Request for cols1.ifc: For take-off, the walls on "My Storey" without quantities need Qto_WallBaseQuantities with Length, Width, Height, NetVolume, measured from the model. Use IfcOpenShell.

First a look at what the model holds.

```python
import ifcopenshell
import ifcopenshell.util.element
import ifcopenshell.util.unit

model = ifcopenshell.open("cols1.ifc")
print(model.schema)
for unit_type in ("LENGTHUNIT", "AREAUNIT", "VOLUMEUNIT"):
    print(unit_type, ifcopenshell.util.unit.calculate_unit_scale(model, unit_type))
storey = next(s for s in model.by_type("IfcBuildingStorey") if s.Name == "My Storey")
walls = [e for e in ifcopenshell.util.element.get_decomposition(storey) if e.is_a("IfcWall")]
for e in sorted(walls, key=lambda e: e.id()):
    print(e.id(), e.is_a(), e.Name, list(ifcopenshell.util.element.get_psets(e, qtos_only=True)), sep=" | ")
```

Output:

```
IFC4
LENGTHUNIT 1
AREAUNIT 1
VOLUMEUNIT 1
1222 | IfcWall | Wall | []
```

```python
import ifcopenshell
import ifcopenshell.api.pset
import ifcopenshell.geom
import ifcopenshell.util.element
import ifcopenshell.util.shape
import ifcopenshell.util.unit

model = ifcopenshell.open("cols1.ifc")
unit_scale = ifcopenshell.util.unit.calculate_unit_scale(model)
volume_scale = ifcopenshell.util.unit.calculate_unit_scale(model, "VOLUMEUNIT")
settings = ifcopenshell.geom.settings()

storey = next(s for s in model.by_type("IfcBuildingStorey") if s.Name == "My Storey")
walls = [e for e in ifcopenshell.util.element.get_decomposition(storey) if e.is_a("IfcWall")]

for e in sorted(walls, key=lambda e: e.id()):
    if ifcopenshell.util.element.get_psets(e, qtos_only=True, should_inherit=False):
        continue
    # Geometry comes back in metres, in the element's own axes.
    shape = ifcopenshell.geom.create_shape(settings, e)
    values = {
        "Length": ifcopenshell.util.shape.get_x(shape.geometry) / unit_scale,
        "Width": ifcopenshell.util.shape.get_y(shape.geometry) / unit_scale,
        "Height": ifcopenshell.util.shape.get_z(shape.geometry) / unit_scale,
        "NetVolume": ifcopenshell.util.shape.get_volume(shape.geometry) / volume_scale,
    }
    qto = ifcopenshell.api.pset.add_qto(model, product=e, name="Qto_WallBaseQuantities")
    ifcopenshell.api.pset.edit_qto(model, qto=qto, properties=values)
    print(e.id(), {k: round(v, 3) for k, v in values.items()})

model.write("cols1_updated.ifc")
```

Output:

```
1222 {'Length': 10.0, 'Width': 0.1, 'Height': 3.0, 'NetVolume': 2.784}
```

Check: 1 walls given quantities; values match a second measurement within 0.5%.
